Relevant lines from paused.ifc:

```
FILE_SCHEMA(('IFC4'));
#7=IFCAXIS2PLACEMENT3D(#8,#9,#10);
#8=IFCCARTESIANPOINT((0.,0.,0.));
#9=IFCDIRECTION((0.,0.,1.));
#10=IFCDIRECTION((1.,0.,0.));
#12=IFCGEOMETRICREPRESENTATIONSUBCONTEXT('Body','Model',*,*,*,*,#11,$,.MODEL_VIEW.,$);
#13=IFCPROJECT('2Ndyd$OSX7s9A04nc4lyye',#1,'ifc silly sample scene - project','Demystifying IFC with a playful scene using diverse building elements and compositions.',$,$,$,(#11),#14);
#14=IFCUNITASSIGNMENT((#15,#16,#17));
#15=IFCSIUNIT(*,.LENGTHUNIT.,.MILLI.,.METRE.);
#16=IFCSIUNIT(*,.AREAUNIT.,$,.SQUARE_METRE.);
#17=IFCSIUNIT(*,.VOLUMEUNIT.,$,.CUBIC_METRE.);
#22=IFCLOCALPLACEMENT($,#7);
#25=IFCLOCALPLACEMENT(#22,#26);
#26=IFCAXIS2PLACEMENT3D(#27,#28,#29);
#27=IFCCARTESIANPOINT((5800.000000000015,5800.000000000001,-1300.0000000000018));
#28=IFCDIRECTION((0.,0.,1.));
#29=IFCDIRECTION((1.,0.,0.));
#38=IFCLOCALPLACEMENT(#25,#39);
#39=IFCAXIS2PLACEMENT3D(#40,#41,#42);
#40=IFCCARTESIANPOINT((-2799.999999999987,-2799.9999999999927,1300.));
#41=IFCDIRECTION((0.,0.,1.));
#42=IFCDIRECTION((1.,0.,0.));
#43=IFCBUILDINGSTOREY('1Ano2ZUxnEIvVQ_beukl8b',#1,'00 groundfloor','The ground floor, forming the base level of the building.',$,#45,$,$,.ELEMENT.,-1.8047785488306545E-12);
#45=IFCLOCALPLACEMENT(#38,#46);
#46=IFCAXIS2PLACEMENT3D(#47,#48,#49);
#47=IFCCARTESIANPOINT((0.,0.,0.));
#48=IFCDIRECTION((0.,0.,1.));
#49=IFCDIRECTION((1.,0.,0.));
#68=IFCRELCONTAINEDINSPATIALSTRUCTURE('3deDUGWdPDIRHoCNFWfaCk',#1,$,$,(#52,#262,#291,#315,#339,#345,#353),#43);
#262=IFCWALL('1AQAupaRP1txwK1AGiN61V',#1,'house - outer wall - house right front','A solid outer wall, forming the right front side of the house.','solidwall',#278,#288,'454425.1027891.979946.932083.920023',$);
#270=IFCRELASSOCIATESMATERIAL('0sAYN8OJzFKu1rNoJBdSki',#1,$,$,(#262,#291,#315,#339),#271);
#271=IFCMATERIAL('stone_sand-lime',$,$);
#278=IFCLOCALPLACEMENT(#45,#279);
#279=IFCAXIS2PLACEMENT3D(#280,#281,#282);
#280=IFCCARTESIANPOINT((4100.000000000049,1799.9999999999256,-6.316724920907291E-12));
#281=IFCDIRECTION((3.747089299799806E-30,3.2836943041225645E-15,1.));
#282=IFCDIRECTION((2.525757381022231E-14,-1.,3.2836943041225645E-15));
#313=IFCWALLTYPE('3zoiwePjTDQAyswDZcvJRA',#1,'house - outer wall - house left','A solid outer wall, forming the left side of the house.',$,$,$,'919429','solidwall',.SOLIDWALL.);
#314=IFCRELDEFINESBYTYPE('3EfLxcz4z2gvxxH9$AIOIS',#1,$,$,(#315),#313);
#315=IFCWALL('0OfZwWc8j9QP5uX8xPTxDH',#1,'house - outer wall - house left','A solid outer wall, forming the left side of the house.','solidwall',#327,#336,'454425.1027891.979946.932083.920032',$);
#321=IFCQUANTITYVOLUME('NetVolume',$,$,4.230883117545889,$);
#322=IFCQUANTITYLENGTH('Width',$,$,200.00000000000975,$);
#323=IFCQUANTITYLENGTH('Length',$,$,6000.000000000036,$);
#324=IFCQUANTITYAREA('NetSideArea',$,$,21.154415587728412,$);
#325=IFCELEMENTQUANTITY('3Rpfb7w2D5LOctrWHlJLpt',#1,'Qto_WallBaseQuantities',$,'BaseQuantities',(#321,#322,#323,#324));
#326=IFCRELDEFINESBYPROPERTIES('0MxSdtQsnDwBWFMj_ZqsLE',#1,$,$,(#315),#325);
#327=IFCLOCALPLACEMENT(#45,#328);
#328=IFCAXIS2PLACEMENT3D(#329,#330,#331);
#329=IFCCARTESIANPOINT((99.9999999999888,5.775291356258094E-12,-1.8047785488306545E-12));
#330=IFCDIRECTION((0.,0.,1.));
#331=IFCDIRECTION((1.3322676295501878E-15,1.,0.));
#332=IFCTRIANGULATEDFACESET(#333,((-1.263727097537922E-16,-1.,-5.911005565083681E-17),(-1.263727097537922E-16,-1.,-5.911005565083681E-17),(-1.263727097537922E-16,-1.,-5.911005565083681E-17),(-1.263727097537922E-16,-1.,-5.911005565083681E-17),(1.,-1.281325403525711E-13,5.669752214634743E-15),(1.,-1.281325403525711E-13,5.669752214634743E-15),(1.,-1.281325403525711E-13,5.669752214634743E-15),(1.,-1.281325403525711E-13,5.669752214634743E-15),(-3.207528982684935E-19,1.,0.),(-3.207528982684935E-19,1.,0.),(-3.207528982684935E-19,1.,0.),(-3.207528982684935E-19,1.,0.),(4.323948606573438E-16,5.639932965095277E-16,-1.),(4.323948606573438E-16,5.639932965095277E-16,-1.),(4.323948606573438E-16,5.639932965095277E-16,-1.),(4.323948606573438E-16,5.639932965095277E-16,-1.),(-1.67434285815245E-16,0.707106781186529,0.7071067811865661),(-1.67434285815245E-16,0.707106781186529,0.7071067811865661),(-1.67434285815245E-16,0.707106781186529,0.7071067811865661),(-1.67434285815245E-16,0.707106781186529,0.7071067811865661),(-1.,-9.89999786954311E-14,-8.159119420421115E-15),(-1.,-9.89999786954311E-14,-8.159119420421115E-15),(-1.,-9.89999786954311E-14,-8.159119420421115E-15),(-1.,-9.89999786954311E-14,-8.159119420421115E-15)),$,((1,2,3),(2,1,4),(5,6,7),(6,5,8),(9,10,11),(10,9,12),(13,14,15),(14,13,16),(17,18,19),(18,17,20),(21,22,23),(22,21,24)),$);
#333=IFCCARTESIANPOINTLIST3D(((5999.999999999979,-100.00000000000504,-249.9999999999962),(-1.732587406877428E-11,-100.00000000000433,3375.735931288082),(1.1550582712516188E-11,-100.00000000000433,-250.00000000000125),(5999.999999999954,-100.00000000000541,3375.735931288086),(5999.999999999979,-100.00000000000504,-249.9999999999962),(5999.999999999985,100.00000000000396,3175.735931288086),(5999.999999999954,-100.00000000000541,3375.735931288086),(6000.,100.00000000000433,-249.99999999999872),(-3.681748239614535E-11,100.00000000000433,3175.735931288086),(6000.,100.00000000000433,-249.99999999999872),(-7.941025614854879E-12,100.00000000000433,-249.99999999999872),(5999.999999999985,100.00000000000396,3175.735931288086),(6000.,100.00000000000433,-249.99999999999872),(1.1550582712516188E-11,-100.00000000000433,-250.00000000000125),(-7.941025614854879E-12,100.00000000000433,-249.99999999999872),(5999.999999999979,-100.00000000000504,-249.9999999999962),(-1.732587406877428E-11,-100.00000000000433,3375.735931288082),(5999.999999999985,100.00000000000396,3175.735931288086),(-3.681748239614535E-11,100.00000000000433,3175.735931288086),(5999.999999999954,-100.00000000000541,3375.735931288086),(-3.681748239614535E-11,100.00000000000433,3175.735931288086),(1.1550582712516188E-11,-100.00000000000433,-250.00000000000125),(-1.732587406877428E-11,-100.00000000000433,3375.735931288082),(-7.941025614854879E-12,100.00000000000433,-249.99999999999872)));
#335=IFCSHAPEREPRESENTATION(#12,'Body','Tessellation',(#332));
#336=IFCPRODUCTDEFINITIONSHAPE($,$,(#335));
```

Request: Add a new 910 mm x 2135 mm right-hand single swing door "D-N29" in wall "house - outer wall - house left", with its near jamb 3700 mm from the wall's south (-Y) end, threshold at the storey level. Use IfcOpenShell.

```python
import numpy as np
import ifcopenshell
import ifcopenshell.api.feature
import ifcopenshell.api.geometry
import ifcopenshell.api.pset
import ifcopenshell.api.root
import ifcopenshell.api.spatial
import ifcopenshell.geom
import ifcopenshell.util.element
import ifcopenshell.util.placement
import ifcopenshell.util.representation
import ifcopenshell.util.shape
import ifcopenshell.util.unit

model = ifcopenshell.open("paused.ifc")
unit_scale = ifcopenshell.util.unit.calculate_unit_scale(model)
area_scale = ifcopenshell.util.unit.calculate_unit_scale(model, "AREAUNIT")
volume_scale = ifcopenshell.util.unit.calculate_unit_scale(model, "VOLUMEUNIT")
settings = ifcopenshell.geom.settings()


def volume(element):
    """Net volume in cubic metres, openings subtracted."""
    shape = ifcopenshell.geom.create_shape(settings, element)
    return ifcopenshell.util.shape.get_volume(shape.geometry)


wall = model.by_guid("0OfZwWc8j9QP5uX8xPTxDH")
storey = ifcopenshell.util.element.get_container(wall, ifc_class="IfcBuildingStorey")
context = ifcopenshell.util.representation.get_context(model, "Model", "Body", "MODEL_VIEW")
before = volume(wall)

width, height, from_end, sill = 0.91, 2.135, 3.7, 0.0  # metres

# The wall runs along its own X axis, and the end named is its -X end.
wall_shape = ifcopenshell.geom.create_shape(settings, wall)
x, y, z = ifcopenshell.util.shape.get_vertices(wall_shape.geometry).T
start = x.min() + from_end
face, thickness = float(y.min()), float(y.max() - y.min())
wall_matrix = ifcopenshell.util.placement.get_local_placement(wall.ObjectPlacement)
level = ifcopenshell.util.placement.get_local_placement(storey.ObjectPlacement)[2, 3]


def in_wall(x, y):
    """Placement at x, y metres in the wall's axes, at sill height."""
    matrix = wall_matrix.copy()
    matrix[:, 3] = wall_matrix @ np.array([x / unit_scale, y / unit_scale, 0.0, 1.0])
    matrix[2, 3] = level + sill / unit_scale
    return matrix


# Opening: a box that overshoots both wall faces by 50 mm.
opening = ifcopenshell.api.root.create_entity(model, ifc_class="IfcOpeningElement", predefined_type="OPENING")
box = ifcopenshell.api.geometry.add_wall_representation(
    model, context=context, length=width, height=height, thickness=thickness + 0.1
)
ifcopenshell.api.geometry.assign_representation(model, product=opening, representation=box)
ifcopenshell.api.geometry.edit_object_placement(model, product=opening, matrix=in_wall(start, face - 0.05), is_si=False)
ifcopenshell.api.feature.add_feature(model, feature=opening, element=wall)

door = ifcopenshell.api.root.create_entity(model, ifc_class="IfcDoor", name="D-N29", predefined_type="DOOR")
door.OverallWidth, door.OverallHeight = width / unit_scale, height / unit_scale
door.OperationType = "SINGLE_SWING_RIGHT"
body = ifcopenshell.api.geometry.add_door_representation(
    model,
    context=context,
    overall_width=door.OverallWidth,
    overall_height=door.OverallHeight,
    operation_type="SINGLE_SWING_RIGHT",
    lining_properties={"LiningDepth": thickness / unit_scale, "ThresholdDepth": thickness / unit_scale},
)
ifcopenshell.api.geometry.assign_representation(model, product=door, representation=body)
ifcopenshell.api.spatial.assign_container(model, products=[door], relating_structure=storey)
ifcopenshell.api.feature.add_filling(model, opening=opening, element=door)

# The lining spans the wall, so the door starts at the wall face.
ifcopenshell.api.geometry.edit_object_placement(model, product=door, matrix=in_wall(start, face), is_si=False)

after = volume(wall)

# Update the wall's stored quantities.
qto = model.by_id(ifcopenshell.util.element.get_pset(wall, "Qto_WallBaseQuantities", should_inherit=False)["id"])
ifcopenshell.api.pset.edit_qto(model, qto=qto, properties={
    "NetVolume": after / volume_scale,
    "NetSideArea": after / thickness / area_scale,
})

print(f"wall volume {before:.3f} -> {after:.3f} m3")

model.write("paused_v2.ifc")
```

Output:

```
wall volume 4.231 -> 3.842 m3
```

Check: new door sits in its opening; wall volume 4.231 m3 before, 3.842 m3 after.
